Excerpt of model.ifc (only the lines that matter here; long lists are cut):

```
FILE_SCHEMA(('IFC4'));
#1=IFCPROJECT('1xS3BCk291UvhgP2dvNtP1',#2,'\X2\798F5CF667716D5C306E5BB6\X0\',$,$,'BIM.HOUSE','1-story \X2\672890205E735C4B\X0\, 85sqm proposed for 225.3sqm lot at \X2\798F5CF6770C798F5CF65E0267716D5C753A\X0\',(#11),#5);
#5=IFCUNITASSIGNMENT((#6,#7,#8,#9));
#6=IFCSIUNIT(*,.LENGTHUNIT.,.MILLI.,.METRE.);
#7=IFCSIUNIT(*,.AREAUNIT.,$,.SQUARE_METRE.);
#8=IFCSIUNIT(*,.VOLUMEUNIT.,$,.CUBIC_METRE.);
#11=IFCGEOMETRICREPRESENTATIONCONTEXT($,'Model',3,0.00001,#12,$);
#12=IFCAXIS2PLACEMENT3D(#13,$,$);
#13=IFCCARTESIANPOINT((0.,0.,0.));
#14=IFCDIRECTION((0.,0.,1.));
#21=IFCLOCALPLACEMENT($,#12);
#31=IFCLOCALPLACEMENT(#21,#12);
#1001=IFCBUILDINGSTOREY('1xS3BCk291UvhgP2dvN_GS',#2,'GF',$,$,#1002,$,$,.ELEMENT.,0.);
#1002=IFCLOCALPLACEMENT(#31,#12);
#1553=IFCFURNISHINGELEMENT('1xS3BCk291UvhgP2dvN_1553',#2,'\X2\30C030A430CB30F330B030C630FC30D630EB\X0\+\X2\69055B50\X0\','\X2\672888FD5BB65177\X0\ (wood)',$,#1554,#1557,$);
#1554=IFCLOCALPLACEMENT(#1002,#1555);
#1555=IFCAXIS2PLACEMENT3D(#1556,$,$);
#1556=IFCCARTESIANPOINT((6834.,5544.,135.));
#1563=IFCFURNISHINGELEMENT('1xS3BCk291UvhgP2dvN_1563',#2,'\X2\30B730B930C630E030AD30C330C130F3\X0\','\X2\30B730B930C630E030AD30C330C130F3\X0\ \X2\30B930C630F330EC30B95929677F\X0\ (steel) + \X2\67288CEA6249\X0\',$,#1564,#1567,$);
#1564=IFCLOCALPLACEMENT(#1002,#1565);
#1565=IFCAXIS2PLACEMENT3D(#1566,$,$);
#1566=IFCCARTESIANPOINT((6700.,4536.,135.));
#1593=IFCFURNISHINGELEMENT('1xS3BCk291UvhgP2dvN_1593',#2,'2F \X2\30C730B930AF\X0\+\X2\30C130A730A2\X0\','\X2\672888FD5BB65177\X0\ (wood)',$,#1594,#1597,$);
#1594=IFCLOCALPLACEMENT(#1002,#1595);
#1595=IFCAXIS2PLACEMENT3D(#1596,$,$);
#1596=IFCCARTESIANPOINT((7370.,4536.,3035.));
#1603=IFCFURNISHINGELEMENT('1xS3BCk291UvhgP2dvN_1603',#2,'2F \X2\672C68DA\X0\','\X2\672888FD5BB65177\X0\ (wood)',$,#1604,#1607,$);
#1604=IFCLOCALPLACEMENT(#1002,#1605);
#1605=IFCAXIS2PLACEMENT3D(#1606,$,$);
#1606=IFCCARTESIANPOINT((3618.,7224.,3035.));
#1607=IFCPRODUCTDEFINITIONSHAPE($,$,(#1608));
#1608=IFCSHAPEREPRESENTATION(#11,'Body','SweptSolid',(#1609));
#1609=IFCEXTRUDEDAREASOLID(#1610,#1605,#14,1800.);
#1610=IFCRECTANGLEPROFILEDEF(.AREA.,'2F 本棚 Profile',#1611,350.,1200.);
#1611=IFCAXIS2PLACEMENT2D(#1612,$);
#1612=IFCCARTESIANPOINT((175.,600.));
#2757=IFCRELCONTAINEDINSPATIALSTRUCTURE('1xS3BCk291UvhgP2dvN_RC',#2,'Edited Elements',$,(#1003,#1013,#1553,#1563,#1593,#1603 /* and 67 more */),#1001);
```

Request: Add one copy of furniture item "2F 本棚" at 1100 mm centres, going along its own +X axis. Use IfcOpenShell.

```python
import ifcopenshell
import ifcopenshell.api.geometry
import ifcopenshell.api.root
import ifcopenshell.util.element
import ifcopenshell.util.placement
import ifcopenshell.util.unit

model = ifcopenshell.open("model.ifc")
unit_scale = ifcopenshell.util.unit.calculate_unit_scale(model)


def reuse_history(source, copy):
    """copy_class also copies each property set's owner history, people and application; keep the originals."""
    for rel in copy.IsDefinedBy:
        if rel.is_a("IfcRelDefinesByProperties") and (history := rel.RelatingPropertyDefinition.OwnerHistory):
            rel.RelatingPropertyDefinition.OwnerHistory = source.OwnerHistory
            ifcopenshell.util.element.remove_deep2(model, history)


source = model.by_id(1603)
base = ifcopenshell.util.placement.get_local_placement(source.ObjectPlacement)
step = base[:3, 0] * 1.1 / unit_scale

for i in range(1, 2):
    copy = ifcopenshell.api.root.copy_class(model, product=source)
    copy.Representation = ifcopenshell.util.element.copy_deep(
        model, source.Representation, exclude=["IfcGeometricRepresentationContext", "IfcRepresentationMap"]
    )
    reuse_history(source, copy)
    matrix = base.copy()
    matrix[:3, 3] += i * step
    print("added at", matrix[:3, 3].round(3) + 0.0)
    ifcopenshell.api.geometry.edit_object_placement(model, product=copy, matrix=matrix, is_si=False)

model.write("model_edited.ifc")
```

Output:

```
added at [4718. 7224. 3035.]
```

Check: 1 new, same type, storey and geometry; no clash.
